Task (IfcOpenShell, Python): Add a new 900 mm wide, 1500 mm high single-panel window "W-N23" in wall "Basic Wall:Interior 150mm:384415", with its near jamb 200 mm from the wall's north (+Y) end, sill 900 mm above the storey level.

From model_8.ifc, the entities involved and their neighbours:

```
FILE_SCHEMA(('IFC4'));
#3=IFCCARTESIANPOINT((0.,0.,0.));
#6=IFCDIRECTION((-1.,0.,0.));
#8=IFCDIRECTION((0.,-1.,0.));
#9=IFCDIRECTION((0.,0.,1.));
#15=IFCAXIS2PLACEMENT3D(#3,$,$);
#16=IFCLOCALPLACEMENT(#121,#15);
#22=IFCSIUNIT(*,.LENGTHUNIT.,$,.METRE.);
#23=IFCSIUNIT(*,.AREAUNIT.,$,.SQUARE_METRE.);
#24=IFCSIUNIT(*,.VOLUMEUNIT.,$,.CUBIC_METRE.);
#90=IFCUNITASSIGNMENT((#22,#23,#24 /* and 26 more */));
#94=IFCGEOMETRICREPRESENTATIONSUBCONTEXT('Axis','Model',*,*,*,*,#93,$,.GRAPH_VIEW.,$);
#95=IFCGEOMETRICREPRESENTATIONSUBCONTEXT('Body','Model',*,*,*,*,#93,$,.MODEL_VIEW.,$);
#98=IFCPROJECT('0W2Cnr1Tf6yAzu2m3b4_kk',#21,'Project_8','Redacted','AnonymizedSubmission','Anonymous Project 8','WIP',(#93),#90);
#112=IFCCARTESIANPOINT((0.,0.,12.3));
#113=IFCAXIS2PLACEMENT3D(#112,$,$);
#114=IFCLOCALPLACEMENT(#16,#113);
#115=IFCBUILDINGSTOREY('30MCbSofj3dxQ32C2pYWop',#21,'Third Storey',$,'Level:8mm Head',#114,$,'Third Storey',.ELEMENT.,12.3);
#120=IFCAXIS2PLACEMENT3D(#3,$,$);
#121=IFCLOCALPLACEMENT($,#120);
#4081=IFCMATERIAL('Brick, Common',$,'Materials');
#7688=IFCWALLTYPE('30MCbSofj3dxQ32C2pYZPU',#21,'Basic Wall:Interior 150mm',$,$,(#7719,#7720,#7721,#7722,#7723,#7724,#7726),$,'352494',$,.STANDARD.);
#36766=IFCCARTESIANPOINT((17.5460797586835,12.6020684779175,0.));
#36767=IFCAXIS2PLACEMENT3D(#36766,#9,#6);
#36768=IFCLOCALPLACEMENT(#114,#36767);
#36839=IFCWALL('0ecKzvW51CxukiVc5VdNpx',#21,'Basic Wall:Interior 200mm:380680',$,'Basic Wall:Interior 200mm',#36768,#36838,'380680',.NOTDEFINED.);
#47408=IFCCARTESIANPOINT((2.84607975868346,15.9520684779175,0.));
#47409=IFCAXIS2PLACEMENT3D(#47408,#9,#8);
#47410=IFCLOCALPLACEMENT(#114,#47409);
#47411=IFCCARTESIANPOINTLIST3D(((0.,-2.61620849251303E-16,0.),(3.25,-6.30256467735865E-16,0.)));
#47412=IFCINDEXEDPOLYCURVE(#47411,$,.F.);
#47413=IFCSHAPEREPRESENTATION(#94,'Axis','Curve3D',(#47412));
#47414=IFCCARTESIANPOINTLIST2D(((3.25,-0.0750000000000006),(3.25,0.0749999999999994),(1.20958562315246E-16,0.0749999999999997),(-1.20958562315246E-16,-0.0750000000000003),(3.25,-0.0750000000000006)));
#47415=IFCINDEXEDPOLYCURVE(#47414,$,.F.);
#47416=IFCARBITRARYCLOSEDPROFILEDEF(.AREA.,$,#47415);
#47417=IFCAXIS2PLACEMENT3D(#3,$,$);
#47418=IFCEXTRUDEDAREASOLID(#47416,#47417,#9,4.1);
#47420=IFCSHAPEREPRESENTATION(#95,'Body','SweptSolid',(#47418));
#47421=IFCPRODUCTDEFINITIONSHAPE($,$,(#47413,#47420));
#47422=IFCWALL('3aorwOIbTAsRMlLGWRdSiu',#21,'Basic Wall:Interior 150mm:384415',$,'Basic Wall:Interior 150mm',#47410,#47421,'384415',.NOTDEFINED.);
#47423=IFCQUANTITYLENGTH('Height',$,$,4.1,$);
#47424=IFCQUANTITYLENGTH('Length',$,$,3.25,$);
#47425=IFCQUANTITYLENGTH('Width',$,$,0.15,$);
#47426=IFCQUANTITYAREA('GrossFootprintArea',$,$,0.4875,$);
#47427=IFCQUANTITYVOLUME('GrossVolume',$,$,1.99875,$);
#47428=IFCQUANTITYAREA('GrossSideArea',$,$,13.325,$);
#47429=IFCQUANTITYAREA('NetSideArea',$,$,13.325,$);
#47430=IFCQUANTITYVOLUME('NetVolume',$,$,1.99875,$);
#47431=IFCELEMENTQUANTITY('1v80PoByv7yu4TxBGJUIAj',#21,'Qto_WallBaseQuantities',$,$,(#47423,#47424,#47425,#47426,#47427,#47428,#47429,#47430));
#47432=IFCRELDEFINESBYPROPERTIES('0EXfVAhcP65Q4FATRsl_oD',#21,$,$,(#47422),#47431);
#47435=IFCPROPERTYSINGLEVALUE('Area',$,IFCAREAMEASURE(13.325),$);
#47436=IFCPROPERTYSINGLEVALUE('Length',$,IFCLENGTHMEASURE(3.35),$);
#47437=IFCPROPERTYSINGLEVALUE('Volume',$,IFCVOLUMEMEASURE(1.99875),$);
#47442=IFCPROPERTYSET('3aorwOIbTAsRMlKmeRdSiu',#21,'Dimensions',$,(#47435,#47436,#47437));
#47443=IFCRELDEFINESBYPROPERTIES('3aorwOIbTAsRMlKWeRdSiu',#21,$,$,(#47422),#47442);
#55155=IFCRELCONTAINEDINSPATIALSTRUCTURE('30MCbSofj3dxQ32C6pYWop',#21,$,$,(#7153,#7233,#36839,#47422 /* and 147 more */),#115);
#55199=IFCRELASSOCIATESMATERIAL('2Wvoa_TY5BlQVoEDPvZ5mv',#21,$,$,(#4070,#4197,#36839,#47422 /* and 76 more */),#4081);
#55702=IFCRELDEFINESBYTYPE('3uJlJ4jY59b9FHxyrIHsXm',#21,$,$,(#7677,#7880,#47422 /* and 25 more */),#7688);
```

```python
import numpy as np
import ifcopenshell
import ifcopenshell.api.feature
import ifcopenshell.api.geometry
import ifcopenshell.api.pset
import ifcopenshell.api.root
import ifcopenshell.api.spatial
import ifcopenshell.geom
import ifcopenshell.util.element
import ifcopenshell.util.placement
import ifcopenshell.util.representation
import ifcopenshell.util.shape
import ifcopenshell.util.unit

model = ifcopenshell.open("model_8.ifc")
unit_scale = ifcopenshell.util.unit.calculate_unit_scale(model)
area_scale = ifcopenshell.util.unit.calculate_unit_scale(model, "AREAUNIT")
volume_scale = ifcopenshell.util.unit.calculate_unit_scale(model, "VOLUMEUNIT")
settings = ifcopenshell.geom.settings()


def volume(element):
    """Net volume in cubic metres, openings subtracted."""
    shape = ifcopenshell.geom.create_shape(settings, element)
    return ifcopenshell.util.shape.get_volume(shape.geometry)


wall = model.by_guid("3aorwOIbTAsRMlLGWRdSiu")
storey = ifcopenshell.util.element.get_container(wall, ifc_class="IfcBuildingStorey")
context = ifcopenshell.util.representation.get_context(model, "Model", "Body", "MODEL_VIEW")
before = volume(wall)

width, height, from_end, sill = 0.9, 1.5, 0.2, 0.9  # metres

# The wall runs along its own X axis, and the end named is its -X end.
wall_shape = ifcopenshell.geom.create_shape(settings, wall)
x, y, z = ifcopenshell.util.shape.get_vertices(wall_shape.geometry).T
start = x.min() + from_end
face, thickness = float(y.min()), float(y.max() - y.min())
wall_matrix = ifcopenshell.util.placement.get_local_placement(wall.ObjectPlacement)
level = ifcopenshell.util.placement.get_local_placement(storey.ObjectPlacement)[2, 3]


def in_wall(x, y):
    """Placement at x, y metres in the wall's axes, at sill height."""
    matrix = wall_matrix.copy()
    matrix[:, 3] = wall_matrix @ np.array([x / unit_scale, y / unit_scale, 0.0, 1.0])
    matrix[2, 3] = level + sill / unit_scale
    return matrix


# Opening: a box that overshoots both wall faces by 50 mm.
opening = ifcopenshell.api.root.create_entity(model, ifc_class="IfcOpeningElement", predefined_type="OPENING")
box = ifcopenshell.api.geometry.add_wall_representation(
    model, context=context, length=width, height=height, thickness=thickness + 0.1
)
ifcopenshell.api.geometry.assign_representation(model, product=opening, representation=box)
ifcopenshell.api.geometry.edit_object_placement(model, product=opening, matrix=in_wall(start, face - 0.05), is_si=False)
ifcopenshell.api.feature.add_feature(model, feature=opening, element=wall)

window = ifcopenshell.api.root.create_entity(model, ifc_class="IfcWindow", name="W-N23", predefined_type="WINDOW")
window.OverallWidth, window.OverallHeight = width / unit_scale, height / unit_scale
window.PartitioningType = "SINGLE_PANEL"
body = ifcopenshell.api.geometry.add_window_representation(
    model,
    context=context,
    overall_width=window.OverallWidth,
    overall_height=window.OverallHeight,
    partition_type="SINGLE_PANEL",
)
ifcopenshell.api.geometry.assign_representation(model, product=window, representation=body)
ifcopenshell.api.spatial.assign_container(model, products=[window], relating_structure=storey)
ifcopenshell.api.feature.add_filling(model, opening=opening, element=window)

# Centre the window in the wall's thickness.
ifcopenshell.api.geometry.edit_object_placement(model, product=window, matrix=in_wall(start, face), is_si=False)
window_shape = ifcopenshell.geom.create_shape(settings, window)
depth = ifcopenshell.util.shape.get_vertices(window_shape.geometry)[:, 1]
offset = face + thickness / 2 - (depth.min() + depth.max()) / 2
ifcopenshell.api.geometry.edit_object_placement(model, product=window, matrix=in_wall(start, offset), is_si=False)

after = volume(wall)

# Update the wall's stored quantities.
qto = model.by_id(ifcopenshell.util.element.get_pset(wall, "Qto_WallBaseQuantities", should_inherit=False)["id"])
ifcopenshell.api.pset.edit_qto(model, qto=qto, properties={
    "NetSideArea": after / thickness / area_scale,
    "NetVolume": after / volume_scale,
})
pset = model.by_id(ifcopenshell.util.element.get_pset(wall, "Dimensions", should_inherit=False)["id"])
ifcopenshell.api.pset.edit_pset(model, pset=pset, properties={
    "Area": model.create_entity("IfcAreaMeasure", after / thickness / area_scale),
    "Volume": model.create_entity("IfcVolumeMeasure", after / volume_scale),
})

print(f"wall volume {before:.3f} -> {after:.3f} m3")

model.write("model_8_updated.ifc")
```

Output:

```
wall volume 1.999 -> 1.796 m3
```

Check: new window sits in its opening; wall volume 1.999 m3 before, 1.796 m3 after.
